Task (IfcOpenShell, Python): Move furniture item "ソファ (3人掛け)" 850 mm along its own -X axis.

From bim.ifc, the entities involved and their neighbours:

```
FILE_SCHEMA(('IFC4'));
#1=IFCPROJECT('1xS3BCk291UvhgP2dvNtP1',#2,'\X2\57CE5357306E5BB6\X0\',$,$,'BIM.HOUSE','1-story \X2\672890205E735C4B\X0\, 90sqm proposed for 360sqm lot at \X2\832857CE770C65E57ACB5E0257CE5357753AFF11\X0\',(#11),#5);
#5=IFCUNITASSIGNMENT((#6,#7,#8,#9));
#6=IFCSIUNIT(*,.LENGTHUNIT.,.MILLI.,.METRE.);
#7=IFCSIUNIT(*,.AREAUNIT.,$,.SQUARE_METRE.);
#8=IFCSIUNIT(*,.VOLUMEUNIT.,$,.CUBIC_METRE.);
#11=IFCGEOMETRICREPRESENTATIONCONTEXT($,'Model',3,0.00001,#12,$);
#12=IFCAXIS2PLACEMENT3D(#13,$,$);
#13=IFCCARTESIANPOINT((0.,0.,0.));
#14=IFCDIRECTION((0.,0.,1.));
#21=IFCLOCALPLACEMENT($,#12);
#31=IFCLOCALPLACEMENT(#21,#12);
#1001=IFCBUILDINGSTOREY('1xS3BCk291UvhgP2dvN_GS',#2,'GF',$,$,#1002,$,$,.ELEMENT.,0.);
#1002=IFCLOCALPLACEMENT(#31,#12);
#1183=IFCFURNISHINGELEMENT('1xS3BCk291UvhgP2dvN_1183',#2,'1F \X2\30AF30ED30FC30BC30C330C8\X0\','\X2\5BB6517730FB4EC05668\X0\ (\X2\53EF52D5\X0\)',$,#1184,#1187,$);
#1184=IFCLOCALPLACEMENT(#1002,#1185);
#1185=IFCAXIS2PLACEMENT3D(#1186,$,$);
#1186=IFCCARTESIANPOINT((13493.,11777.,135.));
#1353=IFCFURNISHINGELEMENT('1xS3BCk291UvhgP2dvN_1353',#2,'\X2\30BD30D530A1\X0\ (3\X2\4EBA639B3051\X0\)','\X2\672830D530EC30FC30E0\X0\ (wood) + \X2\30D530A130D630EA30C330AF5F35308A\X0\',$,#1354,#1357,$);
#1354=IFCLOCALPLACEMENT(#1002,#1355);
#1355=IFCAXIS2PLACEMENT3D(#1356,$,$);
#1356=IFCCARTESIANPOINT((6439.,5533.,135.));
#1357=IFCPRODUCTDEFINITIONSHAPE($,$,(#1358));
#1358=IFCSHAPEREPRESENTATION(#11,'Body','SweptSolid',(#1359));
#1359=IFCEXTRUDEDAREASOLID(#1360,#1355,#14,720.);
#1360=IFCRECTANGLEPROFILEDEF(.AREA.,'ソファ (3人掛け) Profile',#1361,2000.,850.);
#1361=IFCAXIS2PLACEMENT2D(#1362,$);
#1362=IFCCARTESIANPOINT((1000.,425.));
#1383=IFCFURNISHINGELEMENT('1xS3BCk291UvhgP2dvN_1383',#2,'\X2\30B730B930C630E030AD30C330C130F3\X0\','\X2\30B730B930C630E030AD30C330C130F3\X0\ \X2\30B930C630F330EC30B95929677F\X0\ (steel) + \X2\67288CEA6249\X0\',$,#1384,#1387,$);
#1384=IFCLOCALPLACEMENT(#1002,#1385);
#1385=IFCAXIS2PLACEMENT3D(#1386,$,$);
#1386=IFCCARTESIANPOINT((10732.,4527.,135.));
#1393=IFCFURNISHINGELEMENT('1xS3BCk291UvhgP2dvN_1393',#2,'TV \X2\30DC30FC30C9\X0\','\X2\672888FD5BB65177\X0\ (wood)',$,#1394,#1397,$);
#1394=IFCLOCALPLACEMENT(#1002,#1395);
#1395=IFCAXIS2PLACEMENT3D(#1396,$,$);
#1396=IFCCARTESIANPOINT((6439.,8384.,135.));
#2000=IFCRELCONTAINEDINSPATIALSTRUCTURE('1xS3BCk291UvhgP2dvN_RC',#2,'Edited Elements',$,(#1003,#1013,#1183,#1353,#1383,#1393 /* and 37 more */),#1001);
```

```python
import ifcopenshell
import ifcopenshell.api.geometry
import ifcopenshell.util.placement
import ifcopenshell.util.unit

model = ifcopenshell.open("bim.ifc")
unit_scale = ifcopenshell.util.unit.calculate_unit_scale(model)

item = model.by_guid("1xS3BCk291UvhgP2dvN_1353")
matrix = ifcopenshell.util.placement.get_local_placement(item.ObjectPlacement)
matrix[:3, 3] -= matrix[:3, 0] * 0.85 / unit_scale
ifcopenshell.api.geometry.edit_object_placement(model, product=item, matrix=matrix, is_si=False)

print(ifcopenshell.util.placement.get_local_placement(item.ObjectPlacement).round(3) + 0.0)

model.write("bim_v2.ifc")
```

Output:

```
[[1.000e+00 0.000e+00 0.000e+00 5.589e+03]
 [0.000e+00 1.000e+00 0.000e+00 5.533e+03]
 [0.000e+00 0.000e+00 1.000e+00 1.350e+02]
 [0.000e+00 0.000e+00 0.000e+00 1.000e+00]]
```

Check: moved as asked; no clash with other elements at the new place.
